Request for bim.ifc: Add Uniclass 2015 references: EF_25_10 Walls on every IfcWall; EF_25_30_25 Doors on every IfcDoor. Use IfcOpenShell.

First a look at what the model holds.

```python
import ifcopenshell

model = ifcopenshell.open("bim.ifc")
print(model.schema)
print("classifications:", [c.Name for c in model.by_type("IfcClassification")])
for ifc_class in ("IfcDoor", "IfcRoof", "IfcStair", "IfcWall", "IfcWindow"):
    print(ifc_class, len(model.by_type(ifc_class)))
```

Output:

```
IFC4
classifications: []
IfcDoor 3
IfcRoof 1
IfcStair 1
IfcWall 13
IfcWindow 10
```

```python
import ifcopenshell
import ifcopenshell.api.classification

model = ifcopenshell.open("bim.ifc")

system = ifcopenshell.api.classification.add_classification(model, classification="Uniclass 2015")

codes = {
    "IfcWall": ("EF_25_10", "Walls"),
    "IfcDoor": ("EF_25_30_25", "Doors"),
}
for ifc_class, (code, name) in codes.items():
    products = model.by_type(ifc_class)
    ifcopenshell.api.classification.add_reference(
        model, products=products, classification=system, identification=code, name=name
    )
    print(code, len(products))

model.write("bim_v2.ifc")
```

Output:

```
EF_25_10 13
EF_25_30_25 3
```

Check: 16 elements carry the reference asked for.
